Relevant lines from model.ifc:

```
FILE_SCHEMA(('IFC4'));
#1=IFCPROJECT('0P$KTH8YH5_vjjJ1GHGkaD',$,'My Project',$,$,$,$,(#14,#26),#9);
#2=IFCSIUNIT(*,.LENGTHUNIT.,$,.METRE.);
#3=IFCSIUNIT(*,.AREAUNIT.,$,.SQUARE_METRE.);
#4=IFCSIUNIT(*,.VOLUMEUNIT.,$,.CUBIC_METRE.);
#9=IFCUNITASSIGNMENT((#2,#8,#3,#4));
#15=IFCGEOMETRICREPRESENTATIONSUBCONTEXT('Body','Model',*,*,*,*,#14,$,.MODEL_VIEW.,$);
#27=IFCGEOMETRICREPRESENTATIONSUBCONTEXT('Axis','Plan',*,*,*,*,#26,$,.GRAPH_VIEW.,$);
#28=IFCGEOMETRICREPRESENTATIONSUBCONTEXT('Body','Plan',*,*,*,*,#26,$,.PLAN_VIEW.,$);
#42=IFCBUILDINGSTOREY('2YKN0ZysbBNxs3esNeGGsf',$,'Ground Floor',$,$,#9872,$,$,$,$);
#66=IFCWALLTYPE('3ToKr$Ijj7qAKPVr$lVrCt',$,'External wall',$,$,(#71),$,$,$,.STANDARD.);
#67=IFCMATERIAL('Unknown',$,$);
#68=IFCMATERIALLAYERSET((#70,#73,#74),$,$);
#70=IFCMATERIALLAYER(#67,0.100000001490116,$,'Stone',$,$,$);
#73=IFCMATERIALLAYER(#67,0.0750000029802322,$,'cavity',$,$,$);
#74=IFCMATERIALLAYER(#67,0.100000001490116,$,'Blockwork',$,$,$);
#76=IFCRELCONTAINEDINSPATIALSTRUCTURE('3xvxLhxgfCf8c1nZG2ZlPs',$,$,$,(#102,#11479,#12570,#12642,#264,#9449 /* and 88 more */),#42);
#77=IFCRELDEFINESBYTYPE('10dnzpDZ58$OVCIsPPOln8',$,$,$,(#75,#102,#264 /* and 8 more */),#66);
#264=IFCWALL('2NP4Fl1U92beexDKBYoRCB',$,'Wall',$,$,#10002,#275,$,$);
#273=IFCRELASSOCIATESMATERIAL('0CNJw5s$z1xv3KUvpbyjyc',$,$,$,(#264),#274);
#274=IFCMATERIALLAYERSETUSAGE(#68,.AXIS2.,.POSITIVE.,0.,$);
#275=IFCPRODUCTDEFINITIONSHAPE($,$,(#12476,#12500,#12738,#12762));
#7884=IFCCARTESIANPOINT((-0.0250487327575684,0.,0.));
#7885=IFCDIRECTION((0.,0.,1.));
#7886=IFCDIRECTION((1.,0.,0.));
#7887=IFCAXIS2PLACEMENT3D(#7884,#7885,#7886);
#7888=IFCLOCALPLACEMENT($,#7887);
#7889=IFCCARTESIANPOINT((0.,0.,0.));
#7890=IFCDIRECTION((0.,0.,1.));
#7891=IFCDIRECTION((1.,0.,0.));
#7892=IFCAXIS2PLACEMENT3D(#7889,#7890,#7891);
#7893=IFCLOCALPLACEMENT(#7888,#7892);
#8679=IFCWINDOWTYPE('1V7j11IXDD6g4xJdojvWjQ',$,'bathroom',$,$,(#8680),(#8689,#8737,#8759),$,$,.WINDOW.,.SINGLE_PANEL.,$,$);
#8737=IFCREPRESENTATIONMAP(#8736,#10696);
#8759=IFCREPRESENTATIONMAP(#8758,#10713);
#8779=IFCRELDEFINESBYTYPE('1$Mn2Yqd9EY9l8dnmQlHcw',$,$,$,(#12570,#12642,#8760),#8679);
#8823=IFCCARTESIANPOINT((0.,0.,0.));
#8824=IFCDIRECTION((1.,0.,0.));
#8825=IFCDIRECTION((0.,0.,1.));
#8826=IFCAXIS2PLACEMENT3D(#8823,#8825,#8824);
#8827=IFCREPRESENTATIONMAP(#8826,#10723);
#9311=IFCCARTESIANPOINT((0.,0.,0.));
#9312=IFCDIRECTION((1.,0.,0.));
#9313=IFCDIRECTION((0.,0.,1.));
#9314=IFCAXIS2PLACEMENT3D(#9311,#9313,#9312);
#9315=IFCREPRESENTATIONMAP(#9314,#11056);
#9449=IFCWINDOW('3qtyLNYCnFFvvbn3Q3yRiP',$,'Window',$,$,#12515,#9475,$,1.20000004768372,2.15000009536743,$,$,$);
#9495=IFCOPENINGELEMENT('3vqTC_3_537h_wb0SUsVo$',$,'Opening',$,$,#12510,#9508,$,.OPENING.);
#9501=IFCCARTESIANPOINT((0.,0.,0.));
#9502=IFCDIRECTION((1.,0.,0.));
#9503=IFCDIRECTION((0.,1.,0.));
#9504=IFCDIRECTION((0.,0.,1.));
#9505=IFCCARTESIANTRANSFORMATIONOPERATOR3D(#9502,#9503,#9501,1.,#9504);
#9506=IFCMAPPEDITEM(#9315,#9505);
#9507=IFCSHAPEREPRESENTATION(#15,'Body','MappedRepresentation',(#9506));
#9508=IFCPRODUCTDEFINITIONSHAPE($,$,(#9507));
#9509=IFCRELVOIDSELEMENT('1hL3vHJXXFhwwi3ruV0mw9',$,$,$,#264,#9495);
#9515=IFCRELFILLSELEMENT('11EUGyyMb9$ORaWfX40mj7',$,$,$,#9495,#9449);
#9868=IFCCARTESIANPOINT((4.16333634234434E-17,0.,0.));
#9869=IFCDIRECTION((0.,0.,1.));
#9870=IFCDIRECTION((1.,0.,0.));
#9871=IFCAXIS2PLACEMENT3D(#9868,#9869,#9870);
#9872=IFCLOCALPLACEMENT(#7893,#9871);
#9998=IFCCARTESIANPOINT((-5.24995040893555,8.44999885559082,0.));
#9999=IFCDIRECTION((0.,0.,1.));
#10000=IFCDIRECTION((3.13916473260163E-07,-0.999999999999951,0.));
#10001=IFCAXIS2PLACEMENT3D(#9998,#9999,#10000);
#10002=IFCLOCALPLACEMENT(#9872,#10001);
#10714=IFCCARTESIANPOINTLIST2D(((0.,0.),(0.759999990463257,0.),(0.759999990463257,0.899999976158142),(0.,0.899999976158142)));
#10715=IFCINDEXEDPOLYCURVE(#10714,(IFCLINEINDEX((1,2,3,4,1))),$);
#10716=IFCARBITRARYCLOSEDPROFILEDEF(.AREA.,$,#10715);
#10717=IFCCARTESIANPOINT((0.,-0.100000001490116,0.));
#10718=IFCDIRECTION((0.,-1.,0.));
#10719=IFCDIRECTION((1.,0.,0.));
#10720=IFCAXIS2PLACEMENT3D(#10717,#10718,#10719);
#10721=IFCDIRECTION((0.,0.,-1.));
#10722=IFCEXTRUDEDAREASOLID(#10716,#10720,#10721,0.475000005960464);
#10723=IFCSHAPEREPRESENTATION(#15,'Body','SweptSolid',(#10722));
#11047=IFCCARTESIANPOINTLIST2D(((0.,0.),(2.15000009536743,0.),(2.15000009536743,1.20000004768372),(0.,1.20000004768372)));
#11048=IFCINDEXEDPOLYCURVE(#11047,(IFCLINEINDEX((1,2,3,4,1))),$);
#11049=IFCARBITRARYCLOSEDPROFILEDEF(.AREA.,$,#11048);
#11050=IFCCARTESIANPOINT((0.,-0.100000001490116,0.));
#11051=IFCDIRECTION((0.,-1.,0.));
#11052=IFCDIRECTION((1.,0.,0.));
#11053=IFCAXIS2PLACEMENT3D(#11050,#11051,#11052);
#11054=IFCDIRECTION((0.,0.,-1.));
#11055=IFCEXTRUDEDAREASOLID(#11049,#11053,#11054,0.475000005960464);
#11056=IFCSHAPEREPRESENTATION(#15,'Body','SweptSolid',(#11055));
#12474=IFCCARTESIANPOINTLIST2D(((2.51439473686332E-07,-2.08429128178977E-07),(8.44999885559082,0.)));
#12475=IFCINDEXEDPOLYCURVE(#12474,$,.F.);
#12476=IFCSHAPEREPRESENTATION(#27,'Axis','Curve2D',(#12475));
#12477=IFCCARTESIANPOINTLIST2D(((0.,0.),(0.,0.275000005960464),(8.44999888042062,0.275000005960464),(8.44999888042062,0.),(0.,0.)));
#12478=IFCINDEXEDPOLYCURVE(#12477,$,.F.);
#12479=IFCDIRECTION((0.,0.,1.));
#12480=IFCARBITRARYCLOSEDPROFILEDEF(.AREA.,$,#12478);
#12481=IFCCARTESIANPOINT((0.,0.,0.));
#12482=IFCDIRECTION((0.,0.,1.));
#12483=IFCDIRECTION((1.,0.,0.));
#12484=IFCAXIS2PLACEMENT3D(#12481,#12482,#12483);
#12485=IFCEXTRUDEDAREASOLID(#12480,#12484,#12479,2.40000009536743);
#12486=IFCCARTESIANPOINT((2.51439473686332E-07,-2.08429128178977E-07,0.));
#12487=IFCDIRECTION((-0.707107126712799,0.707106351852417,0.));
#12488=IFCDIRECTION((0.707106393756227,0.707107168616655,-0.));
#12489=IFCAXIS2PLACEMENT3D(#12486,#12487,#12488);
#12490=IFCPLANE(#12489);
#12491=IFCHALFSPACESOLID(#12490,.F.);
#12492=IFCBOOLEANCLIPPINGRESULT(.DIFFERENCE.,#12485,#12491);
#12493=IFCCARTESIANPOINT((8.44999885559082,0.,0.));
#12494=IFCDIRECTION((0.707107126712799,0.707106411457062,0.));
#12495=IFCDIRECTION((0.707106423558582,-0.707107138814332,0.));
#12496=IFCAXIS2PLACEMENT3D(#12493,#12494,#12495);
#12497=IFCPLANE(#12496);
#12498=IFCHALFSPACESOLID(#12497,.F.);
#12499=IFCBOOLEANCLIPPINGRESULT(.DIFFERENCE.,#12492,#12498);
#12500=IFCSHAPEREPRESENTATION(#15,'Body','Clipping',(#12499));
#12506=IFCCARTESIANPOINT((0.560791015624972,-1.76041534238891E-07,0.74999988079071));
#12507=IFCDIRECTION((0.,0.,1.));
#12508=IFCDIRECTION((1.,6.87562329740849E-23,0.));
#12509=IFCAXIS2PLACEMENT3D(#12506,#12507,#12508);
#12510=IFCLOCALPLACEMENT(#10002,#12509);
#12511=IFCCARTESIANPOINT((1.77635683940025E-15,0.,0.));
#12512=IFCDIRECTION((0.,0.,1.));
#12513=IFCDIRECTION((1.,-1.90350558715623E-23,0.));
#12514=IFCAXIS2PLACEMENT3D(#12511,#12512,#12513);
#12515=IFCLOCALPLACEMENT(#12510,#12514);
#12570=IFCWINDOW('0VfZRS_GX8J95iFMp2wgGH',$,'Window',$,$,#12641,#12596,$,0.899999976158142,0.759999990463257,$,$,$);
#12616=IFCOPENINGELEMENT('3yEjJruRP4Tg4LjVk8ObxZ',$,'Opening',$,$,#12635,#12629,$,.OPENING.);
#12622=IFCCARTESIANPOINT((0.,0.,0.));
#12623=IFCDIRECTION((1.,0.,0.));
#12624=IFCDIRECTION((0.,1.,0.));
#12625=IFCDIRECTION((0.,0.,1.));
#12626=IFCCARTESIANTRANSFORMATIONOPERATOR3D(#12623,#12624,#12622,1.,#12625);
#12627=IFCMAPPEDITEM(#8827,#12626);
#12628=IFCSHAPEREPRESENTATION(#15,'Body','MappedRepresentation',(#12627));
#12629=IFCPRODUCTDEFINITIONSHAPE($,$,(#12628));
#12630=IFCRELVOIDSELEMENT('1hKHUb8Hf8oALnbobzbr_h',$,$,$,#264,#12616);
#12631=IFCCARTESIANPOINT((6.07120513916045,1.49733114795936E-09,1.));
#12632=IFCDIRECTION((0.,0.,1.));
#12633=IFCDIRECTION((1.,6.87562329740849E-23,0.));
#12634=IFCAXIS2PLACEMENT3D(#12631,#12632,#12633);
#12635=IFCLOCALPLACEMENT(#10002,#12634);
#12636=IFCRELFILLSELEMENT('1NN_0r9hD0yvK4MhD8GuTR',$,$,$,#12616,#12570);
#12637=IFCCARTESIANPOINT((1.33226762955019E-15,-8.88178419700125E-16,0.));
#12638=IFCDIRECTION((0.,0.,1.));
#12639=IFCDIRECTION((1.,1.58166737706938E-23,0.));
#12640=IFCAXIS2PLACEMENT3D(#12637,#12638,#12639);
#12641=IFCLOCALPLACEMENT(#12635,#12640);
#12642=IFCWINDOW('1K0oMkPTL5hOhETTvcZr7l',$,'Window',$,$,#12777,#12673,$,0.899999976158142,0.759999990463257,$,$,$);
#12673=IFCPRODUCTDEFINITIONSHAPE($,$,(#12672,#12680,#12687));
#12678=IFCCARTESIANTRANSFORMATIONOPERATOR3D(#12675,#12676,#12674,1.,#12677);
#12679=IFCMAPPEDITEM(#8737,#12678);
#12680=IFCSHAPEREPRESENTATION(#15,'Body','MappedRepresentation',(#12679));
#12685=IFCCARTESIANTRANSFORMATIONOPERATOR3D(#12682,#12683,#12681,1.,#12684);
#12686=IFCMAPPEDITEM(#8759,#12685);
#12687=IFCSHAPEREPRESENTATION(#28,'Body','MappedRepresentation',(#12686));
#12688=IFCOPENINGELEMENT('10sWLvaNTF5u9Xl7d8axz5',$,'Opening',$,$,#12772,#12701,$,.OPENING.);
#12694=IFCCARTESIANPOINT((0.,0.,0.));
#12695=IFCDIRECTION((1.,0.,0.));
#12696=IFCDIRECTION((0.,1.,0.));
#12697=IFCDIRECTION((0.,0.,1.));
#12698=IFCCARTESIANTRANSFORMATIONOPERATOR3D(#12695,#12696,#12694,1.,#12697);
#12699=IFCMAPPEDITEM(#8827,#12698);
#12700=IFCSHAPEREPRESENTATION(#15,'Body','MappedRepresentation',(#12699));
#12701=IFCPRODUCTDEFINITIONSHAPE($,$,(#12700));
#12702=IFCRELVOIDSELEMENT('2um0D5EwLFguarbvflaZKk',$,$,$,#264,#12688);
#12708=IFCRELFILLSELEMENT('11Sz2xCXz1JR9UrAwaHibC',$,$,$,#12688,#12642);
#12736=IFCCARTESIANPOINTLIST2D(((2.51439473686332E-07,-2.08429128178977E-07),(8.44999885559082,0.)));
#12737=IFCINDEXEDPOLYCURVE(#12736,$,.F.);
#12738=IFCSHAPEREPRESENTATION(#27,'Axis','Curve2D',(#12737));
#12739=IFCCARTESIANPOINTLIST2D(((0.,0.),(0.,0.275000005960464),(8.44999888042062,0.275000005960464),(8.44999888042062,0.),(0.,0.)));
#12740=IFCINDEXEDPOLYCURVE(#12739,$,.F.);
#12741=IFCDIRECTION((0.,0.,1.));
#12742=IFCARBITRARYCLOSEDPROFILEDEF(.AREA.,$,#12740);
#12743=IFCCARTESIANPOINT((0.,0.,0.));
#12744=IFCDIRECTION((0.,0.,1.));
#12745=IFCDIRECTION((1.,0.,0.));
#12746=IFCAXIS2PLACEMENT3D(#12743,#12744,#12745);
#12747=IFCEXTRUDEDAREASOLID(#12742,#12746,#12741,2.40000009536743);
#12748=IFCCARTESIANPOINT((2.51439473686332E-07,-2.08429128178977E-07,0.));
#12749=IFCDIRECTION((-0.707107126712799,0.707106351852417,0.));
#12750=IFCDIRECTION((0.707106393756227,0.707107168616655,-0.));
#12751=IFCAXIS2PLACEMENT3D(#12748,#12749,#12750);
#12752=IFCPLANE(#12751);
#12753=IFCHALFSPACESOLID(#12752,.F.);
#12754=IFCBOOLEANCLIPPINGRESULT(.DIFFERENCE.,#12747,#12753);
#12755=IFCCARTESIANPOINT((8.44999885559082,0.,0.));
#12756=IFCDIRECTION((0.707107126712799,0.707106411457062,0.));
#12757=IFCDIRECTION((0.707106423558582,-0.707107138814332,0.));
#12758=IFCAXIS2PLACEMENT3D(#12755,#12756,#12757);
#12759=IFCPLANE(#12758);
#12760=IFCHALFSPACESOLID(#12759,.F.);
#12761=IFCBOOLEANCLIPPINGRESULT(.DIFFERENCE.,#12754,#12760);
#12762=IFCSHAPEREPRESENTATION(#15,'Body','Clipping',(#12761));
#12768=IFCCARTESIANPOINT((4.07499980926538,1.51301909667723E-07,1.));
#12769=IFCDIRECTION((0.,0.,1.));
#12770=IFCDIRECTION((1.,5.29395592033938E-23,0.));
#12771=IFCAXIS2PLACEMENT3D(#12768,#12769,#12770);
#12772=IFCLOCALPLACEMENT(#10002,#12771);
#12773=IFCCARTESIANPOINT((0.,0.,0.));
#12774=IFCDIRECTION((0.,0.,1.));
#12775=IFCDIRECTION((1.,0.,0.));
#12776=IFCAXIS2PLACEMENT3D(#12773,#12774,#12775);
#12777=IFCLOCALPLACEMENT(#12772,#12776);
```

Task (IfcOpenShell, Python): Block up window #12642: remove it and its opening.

```python
import ifcopenshell
import ifcopenshell.api.feature
import ifcopenshell.api.root
import ifcopenshell.geom
import ifcopenshell.util.shape

model = ifcopenshell.open("model.ifc")
settings = ifcopenshell.geom.settings()


def volume(element):
    """Net volume in cubic metres, openings subtracted."""
    shape = ifcopenshell.geom.create_shape(settings, element)
    return ifcopenshell.util.shape.get_volume(shape.geometry)


window = model.by_id(12642)
opening = window.FillsVoids[0].RelatingOpeningElement
wall = opening.VoidsElements[0].RelatingBuildingElement
before = volume(wall)

ifcopenshell.api.root.remove_product(model, product=window)
ifcopenshell.api.feature.remove_feature(model, feature=opening)

after = volume(wall)

print(f"wall volume {before:.3f} -> {after:.3f} m3")

model.write("model_edited.ifc")
```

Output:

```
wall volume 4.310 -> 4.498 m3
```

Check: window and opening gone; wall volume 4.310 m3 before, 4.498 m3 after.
